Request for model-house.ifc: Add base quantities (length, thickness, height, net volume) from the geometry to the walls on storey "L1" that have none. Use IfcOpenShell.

First a look at what the model holds.

```python
import ifcopenshell
import ifcopenshell.util.element
import ifcopenshell.util.unit

model = ifcopenshell.open("model-house.ifc")
print(model.schema)
for unit_type in ("LENGTHUNIT", "AREAUNIT", "VOLUMEUNIT"):
    print(unit_type, ifcopenshell.util.unit.calculate_unit_scale(model, unit_type))
storey = next(s for s in model.by_type("IfcBuildingStorey") if s.Name == "L1")
walls = [e for e in ifcopenshell.util.element.get_decomposition(storey) if e.is_a("IfcWall")]
for e in sorted(walls, key=lambda e: e.id()):
    print(e.id(), e.is_a(), e.Name, list(ifcopenshell.util.element.get_psets(e, qtos_only=True)), sep=" | ")
```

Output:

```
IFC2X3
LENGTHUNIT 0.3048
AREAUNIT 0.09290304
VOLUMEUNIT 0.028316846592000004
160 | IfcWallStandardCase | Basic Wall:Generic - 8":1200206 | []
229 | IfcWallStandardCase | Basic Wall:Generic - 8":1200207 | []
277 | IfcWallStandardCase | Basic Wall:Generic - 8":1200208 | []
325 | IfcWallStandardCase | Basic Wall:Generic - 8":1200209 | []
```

```python
import ifcopenshell
import ifcopenshell.api.pset
import ifcopenshell.geom
import ifcopenshell.util.element
import ifcopenshell.util.shape
import ifcopenshell.util.unit

model = ifcopenshell.open("model-house.ifc")
unit_scale = ifcopenshell.util.unit.calculate_unit_scale(model)
volume_scale = ifcopenshell.util.unit.calculate_unit_scale(model, "VOLUMEUNIT")
settings = ifcopenshell.geom.settings()

storey = next(s for s in model.by_type("IfcBuildingStorey") if s.Name == "L1")
walls = [e for e in ifcopenshell.util.element.get_decomposition(storey) if e.is_a("IfcWall")]

for e in sorted(walls, key=lambda e: e.id()):
    if ifcopenshell.util.element.get_psets(e, qtos_only=True, should_inherit=False):
        continue
    # Geometry comes back in metres, in the element's own axes.
    shape = ifcopenshell.geom.create_shape(settings, e)
    values = {
        "Length": ifcopenshell.util.shape.get_x(shape.geometry) / unit_scale,
        "Width": ifcopenshell.util.shape.get_y(shape.geometry) / unit_scale,
        "Height": ifcopenshell.util.shape.get_z(shape.geometry) / unit_scale,
        "NetVolume": ifcopenshell.util.shape.get_volume(shape.geometry) / volume_scale,
    }
    qto = ifcopenshell.api.pset.add_qto(model, product=e, name="BaseQuantities")
    ifcopenshell.api.pset.edit_qto(model, qto=qto, properties=values)
    print(e.id(), {k: round(v, 3) for k, v in values.items()})

model.write("model-house_updated.ifc")
```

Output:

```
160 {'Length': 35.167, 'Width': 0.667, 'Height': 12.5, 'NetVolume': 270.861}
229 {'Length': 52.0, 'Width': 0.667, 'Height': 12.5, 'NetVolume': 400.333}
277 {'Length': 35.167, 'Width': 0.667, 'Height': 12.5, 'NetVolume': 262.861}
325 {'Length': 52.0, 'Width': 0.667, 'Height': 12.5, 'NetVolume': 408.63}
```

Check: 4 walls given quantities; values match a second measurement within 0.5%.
